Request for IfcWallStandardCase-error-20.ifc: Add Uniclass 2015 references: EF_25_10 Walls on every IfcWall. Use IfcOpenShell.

First a look at what the model holds.

```python
import ifcopenshell

model = ifcopenshell.open("IfcWallStandardCase-error-20.ifc")
print(model.schema)
print("classifications:", [c.Name for c in model.by_type("IfcClassification")])
for ifc_class in ("IfcDoor", "IfcRoof", "IfcStair", "IfcWall", "IfcWindow"):
    print(ifc_class, len(model.by_type(ifc_class)))
```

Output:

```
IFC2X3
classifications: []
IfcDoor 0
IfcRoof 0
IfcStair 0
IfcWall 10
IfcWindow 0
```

```python
import ifcopenshell
import ifcopenshell.api.classification

model = ifcopenshell.open("IfcWallStandardCase-error-20.ifc")

# IFC2X3 requires Source and Edition and has no link from the project to the system.
system = model.create_entity("IfcClassification", Source="NBS", Edition="2015", Name="Uniclass 2015")

codes = {
    "IfcWall": ("EF_25_10", "Walls"),
}
for ifc_class, (code, name) in codes.items():
    products = model.by_type(ifc_class)
    ifcopenshell.api.classification.add_reference(
        model, products=products, classification=system, identification=code, name=name
    )
    print(code, len(products))

model.write("IfcWallStandardCase-error-20_updated.ifc")
```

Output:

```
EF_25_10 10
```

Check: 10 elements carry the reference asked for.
